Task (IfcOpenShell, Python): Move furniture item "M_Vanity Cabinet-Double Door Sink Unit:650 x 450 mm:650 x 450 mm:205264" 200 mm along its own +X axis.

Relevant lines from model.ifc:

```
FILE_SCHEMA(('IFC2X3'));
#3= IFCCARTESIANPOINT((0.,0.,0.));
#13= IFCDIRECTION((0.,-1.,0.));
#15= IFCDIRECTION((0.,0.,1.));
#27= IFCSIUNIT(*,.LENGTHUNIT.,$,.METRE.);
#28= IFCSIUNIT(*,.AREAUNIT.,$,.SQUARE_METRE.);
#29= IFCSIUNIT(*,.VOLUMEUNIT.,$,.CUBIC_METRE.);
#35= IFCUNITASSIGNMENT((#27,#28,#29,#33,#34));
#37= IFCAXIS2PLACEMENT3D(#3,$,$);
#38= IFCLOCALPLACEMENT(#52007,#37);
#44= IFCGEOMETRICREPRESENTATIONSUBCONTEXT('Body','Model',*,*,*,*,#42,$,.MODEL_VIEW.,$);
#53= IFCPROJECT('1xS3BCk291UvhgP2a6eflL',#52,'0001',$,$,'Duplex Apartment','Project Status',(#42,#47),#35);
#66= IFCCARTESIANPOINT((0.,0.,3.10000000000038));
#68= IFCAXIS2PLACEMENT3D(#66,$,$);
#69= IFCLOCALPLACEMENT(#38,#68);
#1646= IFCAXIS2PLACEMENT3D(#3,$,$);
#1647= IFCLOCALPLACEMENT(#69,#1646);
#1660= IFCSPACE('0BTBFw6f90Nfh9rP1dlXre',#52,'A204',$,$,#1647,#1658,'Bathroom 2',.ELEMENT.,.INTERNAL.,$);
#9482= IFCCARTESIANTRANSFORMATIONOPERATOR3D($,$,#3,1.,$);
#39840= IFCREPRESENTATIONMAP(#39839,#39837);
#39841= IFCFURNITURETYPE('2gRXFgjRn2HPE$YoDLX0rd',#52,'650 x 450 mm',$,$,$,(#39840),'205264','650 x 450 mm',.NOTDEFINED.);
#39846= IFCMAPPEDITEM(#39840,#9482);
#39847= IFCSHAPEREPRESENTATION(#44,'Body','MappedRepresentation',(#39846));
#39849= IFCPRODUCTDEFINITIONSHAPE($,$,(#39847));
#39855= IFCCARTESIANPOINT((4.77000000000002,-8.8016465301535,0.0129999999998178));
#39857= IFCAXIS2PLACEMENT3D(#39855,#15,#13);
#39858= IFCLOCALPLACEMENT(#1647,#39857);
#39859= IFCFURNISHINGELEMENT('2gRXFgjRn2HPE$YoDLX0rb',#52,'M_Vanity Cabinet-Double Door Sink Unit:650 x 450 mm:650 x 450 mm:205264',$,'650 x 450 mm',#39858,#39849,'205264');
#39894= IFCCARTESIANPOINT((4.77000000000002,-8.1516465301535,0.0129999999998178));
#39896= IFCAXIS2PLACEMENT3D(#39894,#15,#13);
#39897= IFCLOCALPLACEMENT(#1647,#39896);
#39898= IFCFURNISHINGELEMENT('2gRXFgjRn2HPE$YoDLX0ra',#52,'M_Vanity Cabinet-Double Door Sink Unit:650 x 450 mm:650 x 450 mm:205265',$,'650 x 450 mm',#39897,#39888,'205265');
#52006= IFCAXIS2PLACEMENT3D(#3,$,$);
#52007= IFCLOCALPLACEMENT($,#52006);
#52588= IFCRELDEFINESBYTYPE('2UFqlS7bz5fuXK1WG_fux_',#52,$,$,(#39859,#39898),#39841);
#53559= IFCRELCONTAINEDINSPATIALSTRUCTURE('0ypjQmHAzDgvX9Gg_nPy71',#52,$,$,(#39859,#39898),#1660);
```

```python
import ifcopenshell
import ifcopenshell.api.geometry
import ifcopenshell.util.placement

model = ifcopenshell.open("model.ifc")

item = model.by_guid("2gRXFgjRn2HPE$YoDLX0rb")
matrix = ifcopenshell.util.placement.get_local_placement(item.ObjectPlacement)
matrix[:3, 3] += matrix[:3, 0] * 0.2
ifcopenshell.api.geometry.edit_object_placement(model, product=item, matrix=matrix, is_si=False)

print(ifcopenshell.util.placement.get_local_placement(item.ObjectPlacement).round(3) + 0.0)

model.write("model_edited.ifc")
```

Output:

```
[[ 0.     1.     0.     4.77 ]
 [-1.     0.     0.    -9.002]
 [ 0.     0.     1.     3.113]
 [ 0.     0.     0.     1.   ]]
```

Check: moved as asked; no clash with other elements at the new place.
